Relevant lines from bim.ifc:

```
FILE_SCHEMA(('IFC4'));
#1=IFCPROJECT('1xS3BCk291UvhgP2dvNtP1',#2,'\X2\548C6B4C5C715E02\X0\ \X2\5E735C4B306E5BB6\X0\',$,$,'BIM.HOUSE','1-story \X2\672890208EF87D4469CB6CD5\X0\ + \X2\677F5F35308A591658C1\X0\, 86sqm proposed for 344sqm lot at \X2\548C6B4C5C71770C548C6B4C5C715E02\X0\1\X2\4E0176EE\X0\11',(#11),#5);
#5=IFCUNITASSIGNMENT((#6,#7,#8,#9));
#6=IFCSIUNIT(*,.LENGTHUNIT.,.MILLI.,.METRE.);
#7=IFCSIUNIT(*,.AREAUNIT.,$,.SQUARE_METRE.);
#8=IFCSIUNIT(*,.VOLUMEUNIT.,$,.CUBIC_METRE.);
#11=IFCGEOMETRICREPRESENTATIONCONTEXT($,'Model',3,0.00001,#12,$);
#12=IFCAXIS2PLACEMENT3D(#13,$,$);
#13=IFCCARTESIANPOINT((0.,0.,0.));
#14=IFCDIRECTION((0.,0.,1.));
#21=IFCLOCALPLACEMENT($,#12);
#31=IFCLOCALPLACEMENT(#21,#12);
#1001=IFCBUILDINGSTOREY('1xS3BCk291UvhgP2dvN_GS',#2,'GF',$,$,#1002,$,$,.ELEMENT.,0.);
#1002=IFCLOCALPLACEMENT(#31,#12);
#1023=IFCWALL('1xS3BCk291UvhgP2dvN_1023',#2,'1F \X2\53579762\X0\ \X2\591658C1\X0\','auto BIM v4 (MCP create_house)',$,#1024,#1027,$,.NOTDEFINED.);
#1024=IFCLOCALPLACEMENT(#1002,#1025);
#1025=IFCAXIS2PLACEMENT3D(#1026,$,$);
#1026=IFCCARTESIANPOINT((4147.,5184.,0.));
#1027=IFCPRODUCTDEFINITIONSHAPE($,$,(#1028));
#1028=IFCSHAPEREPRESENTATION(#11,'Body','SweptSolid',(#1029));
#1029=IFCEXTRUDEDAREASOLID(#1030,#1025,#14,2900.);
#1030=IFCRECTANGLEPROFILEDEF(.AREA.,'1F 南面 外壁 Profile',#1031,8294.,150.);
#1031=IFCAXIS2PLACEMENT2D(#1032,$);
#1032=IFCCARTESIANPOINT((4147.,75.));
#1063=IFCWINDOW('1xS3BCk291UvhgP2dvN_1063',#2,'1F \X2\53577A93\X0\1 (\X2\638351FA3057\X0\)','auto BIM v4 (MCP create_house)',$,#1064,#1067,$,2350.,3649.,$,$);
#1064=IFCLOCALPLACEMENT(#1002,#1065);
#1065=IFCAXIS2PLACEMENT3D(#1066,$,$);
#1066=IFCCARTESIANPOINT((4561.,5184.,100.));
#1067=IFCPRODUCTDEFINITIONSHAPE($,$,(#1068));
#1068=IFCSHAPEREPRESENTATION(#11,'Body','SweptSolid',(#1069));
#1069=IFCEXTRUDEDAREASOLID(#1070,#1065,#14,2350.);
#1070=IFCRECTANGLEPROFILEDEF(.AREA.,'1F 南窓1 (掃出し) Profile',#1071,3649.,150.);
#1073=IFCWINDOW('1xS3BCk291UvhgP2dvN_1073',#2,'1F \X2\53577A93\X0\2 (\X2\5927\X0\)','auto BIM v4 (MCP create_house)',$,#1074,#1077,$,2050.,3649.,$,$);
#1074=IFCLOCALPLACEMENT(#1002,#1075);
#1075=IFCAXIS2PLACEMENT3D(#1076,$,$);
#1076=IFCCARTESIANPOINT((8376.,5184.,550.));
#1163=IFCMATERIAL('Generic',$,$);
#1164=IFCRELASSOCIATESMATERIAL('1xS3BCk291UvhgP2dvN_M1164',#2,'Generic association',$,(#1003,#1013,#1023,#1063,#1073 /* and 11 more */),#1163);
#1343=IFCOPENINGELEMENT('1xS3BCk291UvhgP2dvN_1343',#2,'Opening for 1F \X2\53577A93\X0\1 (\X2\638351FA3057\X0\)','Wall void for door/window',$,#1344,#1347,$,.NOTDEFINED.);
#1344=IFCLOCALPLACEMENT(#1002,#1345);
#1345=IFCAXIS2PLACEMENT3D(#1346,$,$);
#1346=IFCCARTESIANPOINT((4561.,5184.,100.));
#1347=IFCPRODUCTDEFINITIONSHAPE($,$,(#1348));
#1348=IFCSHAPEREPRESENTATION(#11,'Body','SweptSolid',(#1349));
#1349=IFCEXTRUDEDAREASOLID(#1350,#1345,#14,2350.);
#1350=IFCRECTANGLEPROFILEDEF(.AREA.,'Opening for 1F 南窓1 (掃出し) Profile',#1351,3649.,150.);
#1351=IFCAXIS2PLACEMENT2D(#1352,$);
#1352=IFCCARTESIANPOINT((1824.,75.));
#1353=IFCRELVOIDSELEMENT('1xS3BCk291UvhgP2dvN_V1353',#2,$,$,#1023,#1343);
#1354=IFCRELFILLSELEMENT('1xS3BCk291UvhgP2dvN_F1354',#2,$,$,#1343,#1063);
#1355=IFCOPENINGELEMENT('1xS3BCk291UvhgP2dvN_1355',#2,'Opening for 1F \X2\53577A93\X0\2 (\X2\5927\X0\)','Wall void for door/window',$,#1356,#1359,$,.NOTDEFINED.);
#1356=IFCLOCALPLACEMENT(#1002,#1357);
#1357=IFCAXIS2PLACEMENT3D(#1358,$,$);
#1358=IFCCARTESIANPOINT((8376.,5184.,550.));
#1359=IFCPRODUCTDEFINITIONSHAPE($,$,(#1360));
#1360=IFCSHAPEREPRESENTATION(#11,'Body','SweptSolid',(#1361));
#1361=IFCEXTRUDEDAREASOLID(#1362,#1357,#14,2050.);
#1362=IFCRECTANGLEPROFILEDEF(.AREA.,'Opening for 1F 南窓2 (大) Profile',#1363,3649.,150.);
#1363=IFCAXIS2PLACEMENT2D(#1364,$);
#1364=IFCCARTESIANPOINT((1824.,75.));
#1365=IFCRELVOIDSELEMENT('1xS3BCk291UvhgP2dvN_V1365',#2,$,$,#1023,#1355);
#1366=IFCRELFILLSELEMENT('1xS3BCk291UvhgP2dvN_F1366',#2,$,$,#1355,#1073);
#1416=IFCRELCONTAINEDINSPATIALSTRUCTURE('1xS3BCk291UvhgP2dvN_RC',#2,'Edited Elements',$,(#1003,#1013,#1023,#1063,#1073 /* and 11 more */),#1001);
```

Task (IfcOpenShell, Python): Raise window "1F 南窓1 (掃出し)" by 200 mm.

```python
import numpy as np
import ifcopenshell
import ifcopenshell.api.geometry
import ifcopenshell.util.placement
import ifcopenshell.util.unit

model = ifcopenshell.open("bim.ifc")
unit_scale = ifcopenshell.util.unit.calculate_unit_scale(model)

window = model.by_guid("1xS3BCk291UvhgP2dvN_1063")
opening = window.FillsVoids[0].RelatingOpeningElement
dz = 0.2 / unit_scale

shift = np.array([0.0, 0.0, dz])
# The window is not placed relative to its opening, so move both.
for product in (opening, window):
    matrix = ifcopenshell.util.placement.get_local_placement(product.ObjectPlacement)
    matrix[:3, 3] += shift
    ifcopenshell.api.geometry.edit_object_placement(model, product=product, matrix=matrix, is_si=False)

print(f"moved by {dz * unit_scale:+.3f} m")

model.write("bim_updated.ifc")
```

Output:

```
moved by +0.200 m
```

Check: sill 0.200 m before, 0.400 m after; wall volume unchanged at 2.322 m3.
